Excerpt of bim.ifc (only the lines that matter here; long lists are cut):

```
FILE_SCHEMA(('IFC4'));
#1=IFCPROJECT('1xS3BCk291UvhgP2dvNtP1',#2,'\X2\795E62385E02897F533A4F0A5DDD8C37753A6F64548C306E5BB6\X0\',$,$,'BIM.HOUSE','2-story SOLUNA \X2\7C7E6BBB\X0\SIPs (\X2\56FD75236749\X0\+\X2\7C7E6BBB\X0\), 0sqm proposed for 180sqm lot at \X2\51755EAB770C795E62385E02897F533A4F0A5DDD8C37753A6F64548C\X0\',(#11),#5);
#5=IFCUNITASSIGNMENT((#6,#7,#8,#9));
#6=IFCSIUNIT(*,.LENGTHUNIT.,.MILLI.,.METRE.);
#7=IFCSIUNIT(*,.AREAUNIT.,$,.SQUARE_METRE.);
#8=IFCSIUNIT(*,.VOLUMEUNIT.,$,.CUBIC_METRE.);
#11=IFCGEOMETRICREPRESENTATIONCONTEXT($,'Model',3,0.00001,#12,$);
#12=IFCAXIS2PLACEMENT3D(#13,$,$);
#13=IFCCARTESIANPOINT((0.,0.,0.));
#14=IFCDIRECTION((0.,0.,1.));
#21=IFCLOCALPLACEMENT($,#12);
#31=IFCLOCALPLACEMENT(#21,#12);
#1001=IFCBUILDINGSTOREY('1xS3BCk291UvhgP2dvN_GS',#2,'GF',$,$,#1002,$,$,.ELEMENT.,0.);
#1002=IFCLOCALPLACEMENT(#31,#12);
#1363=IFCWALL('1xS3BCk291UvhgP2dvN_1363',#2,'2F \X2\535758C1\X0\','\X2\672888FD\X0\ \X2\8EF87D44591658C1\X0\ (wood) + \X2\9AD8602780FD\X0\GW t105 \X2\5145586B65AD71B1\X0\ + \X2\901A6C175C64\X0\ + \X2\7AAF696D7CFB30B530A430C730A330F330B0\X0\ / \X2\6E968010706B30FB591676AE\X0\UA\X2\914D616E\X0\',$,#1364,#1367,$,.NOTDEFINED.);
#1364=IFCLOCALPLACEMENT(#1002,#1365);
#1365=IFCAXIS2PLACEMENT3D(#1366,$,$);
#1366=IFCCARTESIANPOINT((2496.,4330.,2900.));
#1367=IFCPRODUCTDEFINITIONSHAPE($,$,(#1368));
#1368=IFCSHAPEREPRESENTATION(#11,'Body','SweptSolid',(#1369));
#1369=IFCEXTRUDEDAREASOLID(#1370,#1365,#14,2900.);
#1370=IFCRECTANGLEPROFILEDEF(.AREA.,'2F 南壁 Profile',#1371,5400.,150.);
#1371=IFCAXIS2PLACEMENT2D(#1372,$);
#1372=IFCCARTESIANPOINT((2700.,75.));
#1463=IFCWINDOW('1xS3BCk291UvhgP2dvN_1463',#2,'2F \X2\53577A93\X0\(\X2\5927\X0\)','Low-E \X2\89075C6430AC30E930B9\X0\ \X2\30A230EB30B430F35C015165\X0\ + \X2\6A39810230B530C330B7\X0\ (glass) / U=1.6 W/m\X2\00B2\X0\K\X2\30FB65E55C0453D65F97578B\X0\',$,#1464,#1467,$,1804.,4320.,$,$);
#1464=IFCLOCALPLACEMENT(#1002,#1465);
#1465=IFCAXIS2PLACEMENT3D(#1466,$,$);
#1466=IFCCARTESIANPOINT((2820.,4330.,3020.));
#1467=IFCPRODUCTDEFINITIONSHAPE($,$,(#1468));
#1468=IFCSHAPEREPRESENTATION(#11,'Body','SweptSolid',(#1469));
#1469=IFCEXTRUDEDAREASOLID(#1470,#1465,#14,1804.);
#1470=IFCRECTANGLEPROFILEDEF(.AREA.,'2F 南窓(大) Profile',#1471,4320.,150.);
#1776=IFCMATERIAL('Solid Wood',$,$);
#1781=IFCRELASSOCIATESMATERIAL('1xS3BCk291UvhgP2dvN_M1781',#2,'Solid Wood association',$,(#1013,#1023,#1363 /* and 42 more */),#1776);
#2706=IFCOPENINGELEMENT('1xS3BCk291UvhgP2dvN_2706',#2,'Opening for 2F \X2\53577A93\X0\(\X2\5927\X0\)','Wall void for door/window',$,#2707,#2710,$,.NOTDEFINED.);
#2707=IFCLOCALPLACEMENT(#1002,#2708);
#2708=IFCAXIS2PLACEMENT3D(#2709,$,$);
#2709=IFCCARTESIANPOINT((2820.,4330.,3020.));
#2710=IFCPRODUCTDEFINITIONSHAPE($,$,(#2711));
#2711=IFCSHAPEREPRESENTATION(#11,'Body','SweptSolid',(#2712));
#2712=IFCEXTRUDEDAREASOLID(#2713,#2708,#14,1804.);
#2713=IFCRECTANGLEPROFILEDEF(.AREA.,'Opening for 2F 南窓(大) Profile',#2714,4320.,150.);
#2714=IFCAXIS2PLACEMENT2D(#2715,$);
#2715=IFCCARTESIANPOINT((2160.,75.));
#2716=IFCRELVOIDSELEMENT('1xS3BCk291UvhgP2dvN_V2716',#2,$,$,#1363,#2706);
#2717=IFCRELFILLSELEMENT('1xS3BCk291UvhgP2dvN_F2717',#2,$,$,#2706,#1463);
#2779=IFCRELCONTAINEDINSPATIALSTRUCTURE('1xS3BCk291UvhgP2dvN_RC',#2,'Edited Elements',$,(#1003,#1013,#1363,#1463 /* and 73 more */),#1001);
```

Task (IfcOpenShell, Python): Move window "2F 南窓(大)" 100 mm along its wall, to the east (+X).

```python
import ifcopenshell
import ifcopenshell.api.geometry
import ifcopenshell.util.placement
import ifcopenshell.util.unit

model = ifcopenshell.open("bim.ifc")
unit_scale = ifcopenshell.util.unit.calculate_unit_scale(model)

window = model.by_guid("1xS3BCk291UvhgP2dvN_1463")
opening = window.FillsVoids[0].RelatingOpeningElement
wall = opening.VoidsElements[0].RelatingBuildingElement

wall_matrix = ifcopenshell.util.placement.get_local_placement(wall.ObjectPlacement)
shift = wall_matrix[:3, 0] * 0.1 / unit_scale
before = ifcopenshell.util.placement.get_local_placement(window.ObjectPlacement)[:3, 3].copy()

# The window is not placed relative to its opening, so move both.
for product in (opening, window):
    matrix = ifcopenshell.util.placement.get_local_placement(product.ObjectPlacement)
    matrix[:3, 3] += shift
    ifcopenshell.api.geometry.edit_object_placement(model, product=product, matrix=matrix, is_si=False)

after = ifcopenshell.util.placement.get_local_placement(window.ObjectPlacement)[:3, 3]
print("window moved by", (after - before).round(3) + 0.0)

model.write("bim_edited.ifc")
```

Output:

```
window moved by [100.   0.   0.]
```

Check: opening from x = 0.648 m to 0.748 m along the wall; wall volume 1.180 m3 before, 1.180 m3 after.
